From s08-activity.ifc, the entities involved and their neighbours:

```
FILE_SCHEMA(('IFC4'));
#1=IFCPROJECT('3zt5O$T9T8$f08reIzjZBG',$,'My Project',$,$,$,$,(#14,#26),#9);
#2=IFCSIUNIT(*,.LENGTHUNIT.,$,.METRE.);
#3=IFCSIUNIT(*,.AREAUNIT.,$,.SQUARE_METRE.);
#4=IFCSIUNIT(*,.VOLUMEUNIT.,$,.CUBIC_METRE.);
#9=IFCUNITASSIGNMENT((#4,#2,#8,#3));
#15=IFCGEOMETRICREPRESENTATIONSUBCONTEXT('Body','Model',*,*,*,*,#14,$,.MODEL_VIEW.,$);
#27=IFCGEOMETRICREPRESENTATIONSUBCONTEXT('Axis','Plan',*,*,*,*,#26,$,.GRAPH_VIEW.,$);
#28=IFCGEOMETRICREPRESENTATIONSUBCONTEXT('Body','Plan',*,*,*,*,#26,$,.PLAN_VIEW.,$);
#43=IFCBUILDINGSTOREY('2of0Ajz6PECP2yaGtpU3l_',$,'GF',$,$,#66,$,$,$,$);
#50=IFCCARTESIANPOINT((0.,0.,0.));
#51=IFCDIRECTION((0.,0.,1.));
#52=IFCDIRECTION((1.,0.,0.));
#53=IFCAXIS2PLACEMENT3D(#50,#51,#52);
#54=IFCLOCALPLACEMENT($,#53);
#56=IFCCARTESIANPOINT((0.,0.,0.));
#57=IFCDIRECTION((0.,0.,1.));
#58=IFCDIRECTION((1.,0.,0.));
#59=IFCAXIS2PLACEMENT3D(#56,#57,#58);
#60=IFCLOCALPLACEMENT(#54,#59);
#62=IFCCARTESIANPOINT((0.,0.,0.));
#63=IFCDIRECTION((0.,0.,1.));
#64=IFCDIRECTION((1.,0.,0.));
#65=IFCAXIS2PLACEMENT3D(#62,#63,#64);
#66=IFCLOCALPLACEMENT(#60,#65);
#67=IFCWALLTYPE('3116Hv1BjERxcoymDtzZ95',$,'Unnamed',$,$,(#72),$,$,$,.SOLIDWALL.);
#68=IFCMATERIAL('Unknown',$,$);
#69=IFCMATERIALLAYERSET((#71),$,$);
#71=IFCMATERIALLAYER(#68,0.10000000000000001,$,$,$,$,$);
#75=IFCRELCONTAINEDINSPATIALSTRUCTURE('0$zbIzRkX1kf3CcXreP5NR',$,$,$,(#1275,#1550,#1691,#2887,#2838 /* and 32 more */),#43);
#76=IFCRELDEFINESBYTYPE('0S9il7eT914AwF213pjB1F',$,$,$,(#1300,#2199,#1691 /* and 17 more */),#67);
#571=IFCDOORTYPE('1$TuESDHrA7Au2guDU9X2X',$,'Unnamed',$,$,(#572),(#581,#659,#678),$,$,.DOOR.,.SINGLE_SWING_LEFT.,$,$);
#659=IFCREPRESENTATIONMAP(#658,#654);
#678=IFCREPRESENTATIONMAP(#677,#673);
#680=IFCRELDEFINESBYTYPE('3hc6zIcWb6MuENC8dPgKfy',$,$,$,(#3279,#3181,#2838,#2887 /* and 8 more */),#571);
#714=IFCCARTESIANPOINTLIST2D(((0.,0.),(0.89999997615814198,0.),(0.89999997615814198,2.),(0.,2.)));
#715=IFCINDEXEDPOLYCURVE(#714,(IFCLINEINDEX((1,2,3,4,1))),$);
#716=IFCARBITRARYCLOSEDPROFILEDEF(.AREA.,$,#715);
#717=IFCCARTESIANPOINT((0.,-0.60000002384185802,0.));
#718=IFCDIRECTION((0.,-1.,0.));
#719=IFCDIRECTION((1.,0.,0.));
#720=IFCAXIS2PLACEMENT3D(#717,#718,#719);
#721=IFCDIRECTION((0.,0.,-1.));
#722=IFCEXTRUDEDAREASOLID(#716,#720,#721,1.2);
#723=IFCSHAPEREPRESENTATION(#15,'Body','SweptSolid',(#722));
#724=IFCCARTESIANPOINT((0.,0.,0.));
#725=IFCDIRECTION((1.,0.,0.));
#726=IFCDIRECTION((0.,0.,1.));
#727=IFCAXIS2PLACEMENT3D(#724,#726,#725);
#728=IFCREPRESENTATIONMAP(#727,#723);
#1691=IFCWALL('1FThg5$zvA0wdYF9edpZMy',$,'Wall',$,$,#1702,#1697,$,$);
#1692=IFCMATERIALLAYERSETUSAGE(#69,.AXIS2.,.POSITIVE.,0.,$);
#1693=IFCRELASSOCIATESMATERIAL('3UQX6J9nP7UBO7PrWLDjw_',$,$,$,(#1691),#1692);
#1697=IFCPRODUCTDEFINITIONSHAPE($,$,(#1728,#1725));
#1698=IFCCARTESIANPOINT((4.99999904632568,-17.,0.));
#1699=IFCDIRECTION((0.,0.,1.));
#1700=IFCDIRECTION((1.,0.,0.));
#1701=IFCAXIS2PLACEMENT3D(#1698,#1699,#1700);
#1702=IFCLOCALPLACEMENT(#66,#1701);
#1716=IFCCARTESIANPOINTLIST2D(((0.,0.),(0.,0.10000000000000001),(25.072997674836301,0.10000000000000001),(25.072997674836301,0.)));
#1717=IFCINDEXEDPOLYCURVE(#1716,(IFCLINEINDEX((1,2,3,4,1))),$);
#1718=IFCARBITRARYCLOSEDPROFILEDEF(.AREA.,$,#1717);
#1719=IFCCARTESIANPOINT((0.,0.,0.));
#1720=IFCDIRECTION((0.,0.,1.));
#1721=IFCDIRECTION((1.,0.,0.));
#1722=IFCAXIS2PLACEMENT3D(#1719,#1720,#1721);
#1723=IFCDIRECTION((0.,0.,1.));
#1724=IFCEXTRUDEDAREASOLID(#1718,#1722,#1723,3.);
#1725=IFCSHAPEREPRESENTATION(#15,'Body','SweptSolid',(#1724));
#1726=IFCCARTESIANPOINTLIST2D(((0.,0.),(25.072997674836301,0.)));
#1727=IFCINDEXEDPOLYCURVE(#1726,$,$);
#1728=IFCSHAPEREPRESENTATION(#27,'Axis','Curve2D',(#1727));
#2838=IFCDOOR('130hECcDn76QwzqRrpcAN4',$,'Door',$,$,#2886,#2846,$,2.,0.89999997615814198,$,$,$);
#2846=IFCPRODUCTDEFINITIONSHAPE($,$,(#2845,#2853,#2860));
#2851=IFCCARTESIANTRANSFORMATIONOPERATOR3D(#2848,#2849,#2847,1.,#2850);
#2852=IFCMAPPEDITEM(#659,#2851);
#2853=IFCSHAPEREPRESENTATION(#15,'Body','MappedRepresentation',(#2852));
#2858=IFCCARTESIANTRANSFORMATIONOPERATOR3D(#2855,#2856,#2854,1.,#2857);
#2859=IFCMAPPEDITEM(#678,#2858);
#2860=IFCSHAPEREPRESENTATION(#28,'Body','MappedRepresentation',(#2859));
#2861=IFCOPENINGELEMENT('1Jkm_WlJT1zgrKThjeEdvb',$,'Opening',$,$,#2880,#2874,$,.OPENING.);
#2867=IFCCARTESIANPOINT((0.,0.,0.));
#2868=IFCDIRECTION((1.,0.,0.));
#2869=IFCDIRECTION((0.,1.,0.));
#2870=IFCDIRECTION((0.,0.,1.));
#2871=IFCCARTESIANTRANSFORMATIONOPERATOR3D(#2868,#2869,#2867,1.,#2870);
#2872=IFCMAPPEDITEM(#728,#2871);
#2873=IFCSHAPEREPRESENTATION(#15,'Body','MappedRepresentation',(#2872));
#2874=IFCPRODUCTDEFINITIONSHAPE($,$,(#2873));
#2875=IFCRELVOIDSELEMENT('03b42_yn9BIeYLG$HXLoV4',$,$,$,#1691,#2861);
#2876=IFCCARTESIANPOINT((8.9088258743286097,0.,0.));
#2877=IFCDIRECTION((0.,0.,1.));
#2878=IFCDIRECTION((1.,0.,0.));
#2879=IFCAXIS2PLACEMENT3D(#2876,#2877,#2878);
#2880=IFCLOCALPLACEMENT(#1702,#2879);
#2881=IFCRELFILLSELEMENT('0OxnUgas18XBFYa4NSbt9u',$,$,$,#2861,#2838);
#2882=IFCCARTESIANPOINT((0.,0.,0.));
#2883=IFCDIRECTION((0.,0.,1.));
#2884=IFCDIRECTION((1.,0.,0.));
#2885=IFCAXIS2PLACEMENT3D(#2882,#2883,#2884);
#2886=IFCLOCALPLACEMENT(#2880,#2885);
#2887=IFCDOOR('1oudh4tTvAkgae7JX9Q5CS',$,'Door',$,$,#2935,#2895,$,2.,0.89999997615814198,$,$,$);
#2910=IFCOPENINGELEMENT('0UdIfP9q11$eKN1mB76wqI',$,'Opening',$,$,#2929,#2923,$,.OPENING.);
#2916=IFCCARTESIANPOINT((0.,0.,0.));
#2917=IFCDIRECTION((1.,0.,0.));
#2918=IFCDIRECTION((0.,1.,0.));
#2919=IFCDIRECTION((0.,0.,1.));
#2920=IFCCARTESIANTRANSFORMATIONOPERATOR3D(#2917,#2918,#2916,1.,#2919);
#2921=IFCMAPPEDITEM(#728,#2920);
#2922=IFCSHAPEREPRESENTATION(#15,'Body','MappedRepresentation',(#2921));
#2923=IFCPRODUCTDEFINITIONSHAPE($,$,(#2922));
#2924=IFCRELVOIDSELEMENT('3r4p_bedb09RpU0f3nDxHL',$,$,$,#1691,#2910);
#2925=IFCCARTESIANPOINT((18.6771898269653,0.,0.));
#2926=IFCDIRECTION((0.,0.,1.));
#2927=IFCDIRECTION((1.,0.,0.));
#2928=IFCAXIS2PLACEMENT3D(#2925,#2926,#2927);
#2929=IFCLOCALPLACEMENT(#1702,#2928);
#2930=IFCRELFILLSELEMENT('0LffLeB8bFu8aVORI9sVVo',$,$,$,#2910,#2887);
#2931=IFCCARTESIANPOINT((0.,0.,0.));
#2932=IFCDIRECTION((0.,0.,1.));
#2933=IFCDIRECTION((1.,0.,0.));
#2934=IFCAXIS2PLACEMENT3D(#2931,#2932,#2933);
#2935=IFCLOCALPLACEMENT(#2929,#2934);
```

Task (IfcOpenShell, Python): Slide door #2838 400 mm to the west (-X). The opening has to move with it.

```python
import ifcopenshell
import ifcopenshell.api.geometry
import ifcopenshell.util.placement

model = ifcopenshell.open("s08-activity.ifc")

door = model.by_guid("130hECcDn76QwzqRrpcAN4")
opening = door.FillsVoids[0].RelatingOpeningElement
wall = opening.VoidsElements[0].RelatingBuildingElement

wall_matrix = ifcopenshell.util.placement.get_local_placement(wall.ObjectPlacement)
shift = wall_matrix[:3, 0] * -0.4
before = ifcopenshell.util.placement.get_local_placement(door.ObjectPlacement)[:3, 3].copy()

# The door is placed relative to its opening, so it follows when the opening moves.
matrix = ifcopenshell.util.placement.get_local_placement(opening.ObjectPlacement)
matrix[:3, 3] += shift
ifcopenshell.api.geometry.edit_object_placement(
    model, product=opening, matrix=matrix, is_si=False, should_transform_children=True
)

after = ifcopenshell.util.placement.get_local_placement(door.ObjectPlacement)[:3, 3]
print("door moved by", (after - before).round(3) + 0.0)

model.write("s08-activity_edited.ifc")
```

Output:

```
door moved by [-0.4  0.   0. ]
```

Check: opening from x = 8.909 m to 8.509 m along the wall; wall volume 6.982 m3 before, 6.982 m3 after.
